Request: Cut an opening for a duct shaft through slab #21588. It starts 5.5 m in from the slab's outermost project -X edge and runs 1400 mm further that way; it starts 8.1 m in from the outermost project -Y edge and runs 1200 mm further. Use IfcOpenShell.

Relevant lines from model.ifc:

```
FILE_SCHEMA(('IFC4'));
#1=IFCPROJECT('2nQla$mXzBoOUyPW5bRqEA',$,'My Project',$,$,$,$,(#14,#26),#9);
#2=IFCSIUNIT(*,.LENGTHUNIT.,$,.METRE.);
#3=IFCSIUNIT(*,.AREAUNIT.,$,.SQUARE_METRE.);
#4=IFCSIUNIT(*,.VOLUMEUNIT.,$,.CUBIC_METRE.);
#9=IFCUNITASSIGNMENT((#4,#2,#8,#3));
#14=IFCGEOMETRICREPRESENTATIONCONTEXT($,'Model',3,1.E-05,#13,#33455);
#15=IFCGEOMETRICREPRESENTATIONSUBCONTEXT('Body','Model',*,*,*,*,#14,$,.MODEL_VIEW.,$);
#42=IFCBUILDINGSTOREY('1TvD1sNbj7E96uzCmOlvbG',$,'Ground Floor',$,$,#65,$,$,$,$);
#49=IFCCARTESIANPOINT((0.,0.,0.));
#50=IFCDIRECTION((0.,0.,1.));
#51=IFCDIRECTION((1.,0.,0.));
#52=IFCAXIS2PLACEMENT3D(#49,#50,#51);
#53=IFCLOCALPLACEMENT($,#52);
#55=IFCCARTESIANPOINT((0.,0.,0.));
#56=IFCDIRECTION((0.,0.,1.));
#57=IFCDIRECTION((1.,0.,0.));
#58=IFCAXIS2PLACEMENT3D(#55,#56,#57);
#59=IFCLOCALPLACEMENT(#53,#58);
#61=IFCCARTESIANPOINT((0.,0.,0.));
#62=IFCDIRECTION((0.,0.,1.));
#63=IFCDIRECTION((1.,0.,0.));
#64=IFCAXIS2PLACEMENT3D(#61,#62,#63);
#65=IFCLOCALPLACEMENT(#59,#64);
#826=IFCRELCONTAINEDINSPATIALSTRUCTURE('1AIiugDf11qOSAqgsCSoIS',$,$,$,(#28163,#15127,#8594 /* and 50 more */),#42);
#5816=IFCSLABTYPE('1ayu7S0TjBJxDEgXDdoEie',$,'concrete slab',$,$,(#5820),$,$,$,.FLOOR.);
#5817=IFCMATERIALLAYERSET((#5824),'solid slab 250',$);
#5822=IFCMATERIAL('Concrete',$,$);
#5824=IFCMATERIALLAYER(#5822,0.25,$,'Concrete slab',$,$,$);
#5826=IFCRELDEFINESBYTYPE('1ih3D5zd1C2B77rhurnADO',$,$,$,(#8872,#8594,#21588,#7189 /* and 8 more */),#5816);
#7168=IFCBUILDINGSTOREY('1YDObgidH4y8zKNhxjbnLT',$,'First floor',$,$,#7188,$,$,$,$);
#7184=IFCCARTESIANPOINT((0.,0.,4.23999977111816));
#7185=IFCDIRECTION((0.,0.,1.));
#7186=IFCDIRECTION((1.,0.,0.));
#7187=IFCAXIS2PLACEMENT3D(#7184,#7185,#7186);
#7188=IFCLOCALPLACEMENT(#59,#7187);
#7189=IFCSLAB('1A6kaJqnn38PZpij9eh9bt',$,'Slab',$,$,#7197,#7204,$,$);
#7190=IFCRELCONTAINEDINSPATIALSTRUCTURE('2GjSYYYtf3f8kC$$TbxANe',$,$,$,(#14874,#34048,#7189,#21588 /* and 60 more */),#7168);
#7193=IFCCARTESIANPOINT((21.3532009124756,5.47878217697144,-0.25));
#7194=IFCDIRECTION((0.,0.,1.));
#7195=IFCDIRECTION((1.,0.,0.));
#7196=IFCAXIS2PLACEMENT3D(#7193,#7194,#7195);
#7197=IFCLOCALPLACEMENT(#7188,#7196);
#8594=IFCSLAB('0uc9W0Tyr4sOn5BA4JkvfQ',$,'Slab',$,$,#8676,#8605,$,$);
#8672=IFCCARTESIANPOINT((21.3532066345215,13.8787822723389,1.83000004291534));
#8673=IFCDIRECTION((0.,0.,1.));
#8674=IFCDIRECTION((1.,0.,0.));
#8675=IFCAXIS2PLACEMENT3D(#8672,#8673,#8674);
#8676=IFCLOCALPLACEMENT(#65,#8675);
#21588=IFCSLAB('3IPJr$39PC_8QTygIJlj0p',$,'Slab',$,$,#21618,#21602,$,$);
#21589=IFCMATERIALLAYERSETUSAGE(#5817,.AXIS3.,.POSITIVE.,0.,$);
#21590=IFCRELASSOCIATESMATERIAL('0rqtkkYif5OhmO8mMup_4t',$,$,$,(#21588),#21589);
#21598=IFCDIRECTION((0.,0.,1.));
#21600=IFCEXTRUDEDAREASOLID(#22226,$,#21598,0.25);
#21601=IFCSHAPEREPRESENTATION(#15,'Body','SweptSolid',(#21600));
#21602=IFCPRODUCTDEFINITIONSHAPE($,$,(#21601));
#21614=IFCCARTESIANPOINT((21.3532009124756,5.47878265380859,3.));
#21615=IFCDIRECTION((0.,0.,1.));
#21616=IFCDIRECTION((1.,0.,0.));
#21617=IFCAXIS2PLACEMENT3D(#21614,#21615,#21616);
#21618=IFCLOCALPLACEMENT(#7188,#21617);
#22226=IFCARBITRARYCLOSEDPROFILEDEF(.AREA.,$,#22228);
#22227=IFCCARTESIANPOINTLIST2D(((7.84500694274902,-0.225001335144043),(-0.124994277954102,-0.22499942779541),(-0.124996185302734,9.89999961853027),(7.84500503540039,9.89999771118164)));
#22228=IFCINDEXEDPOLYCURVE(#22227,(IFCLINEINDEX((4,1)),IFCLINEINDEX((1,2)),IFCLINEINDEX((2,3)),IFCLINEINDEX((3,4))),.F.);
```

```python
import numpy as np
import ifcopenshell
import ifcopenshell.api.feature
import ifcopenshell.api.geometry
import ifcopenshell.api.root
import ifcopenshell.geom
import ifcopenshell.util.placement
import ifcopenshell.util.representation
import ifcopenshell.util.shape
import ifcopenshell.util.unit

model = ifcopenshell.open("model.ifc")
unit_scale = ifcopenshell.util.unit.calculate_unit_scale(model)
settings = ifcopenshell.geom.settings()


def volume(element):
    """Net volume in cubic metres, openings subtracted."""
    shape = ifcopenshell.geom.create_shape(settings, element)
    return ifcopenshell.util.shape.get_volume(shape.geometry)


slab = model.by_id(21588)
before = volume(slab)

# Extent in the slab's own axes, in metres. The edges named are its -X and -Y sides.
slab_shape = ifcopenshell.geom.create_shape(settings, slab)
vertices = ifcopenshell.util.shape.get_vertices(slab_shape.geometry)
x_min, y_min, bottom = vertices.min(axis=0)
top = vertices[:, 2].max()

opening = ifcopenshell.api.root.create_entity(model, ifc_class="IfcOpeningElement", name="Duct shaft opening", predefined_type="OPENING")
context = ifcopenshell.util.representation.get_context(model, "Model", "Body", "MODEL_VIEW")
width, depth = 1.4, 1.2
outline = [(0.0, 0.0), (width, 0.0), (width, depth), (0.0, depth), (0.0, 0.0)]
# Overshoot both faces by 50 mm so the cut is clean.
shape = ifcopenshell.api.geometry.add_slab_representation(
    model, context=context, depth=top - bottom + 0.1, polyline=outline
)
ifcopenshell.api.geometry.assign_representation(model, product=opening, representation=shape)

matrix = ifcopenshell.util.placement.get_local_placement(slab.ObjectPlacement)
matrix[:, 3] = matrix @ np.append(np.array([x_min + 5.5, y_min + 8.1, bottom - 0.05]) / unit_scale, 1.0)
ifcopenshell.api.geometry.edit_object_placement(model, product=opening, matrix=matrix, is_si=False)
ifcopenshell.api.feature.add_feature(model, feature=opening, element=slab)

after = volume(slab)

print(f"slab volume {before:.3f} -> {after:.3f} m3")

model.write("model_updated.ifc")
```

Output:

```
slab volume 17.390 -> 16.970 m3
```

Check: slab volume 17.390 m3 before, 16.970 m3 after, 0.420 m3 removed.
